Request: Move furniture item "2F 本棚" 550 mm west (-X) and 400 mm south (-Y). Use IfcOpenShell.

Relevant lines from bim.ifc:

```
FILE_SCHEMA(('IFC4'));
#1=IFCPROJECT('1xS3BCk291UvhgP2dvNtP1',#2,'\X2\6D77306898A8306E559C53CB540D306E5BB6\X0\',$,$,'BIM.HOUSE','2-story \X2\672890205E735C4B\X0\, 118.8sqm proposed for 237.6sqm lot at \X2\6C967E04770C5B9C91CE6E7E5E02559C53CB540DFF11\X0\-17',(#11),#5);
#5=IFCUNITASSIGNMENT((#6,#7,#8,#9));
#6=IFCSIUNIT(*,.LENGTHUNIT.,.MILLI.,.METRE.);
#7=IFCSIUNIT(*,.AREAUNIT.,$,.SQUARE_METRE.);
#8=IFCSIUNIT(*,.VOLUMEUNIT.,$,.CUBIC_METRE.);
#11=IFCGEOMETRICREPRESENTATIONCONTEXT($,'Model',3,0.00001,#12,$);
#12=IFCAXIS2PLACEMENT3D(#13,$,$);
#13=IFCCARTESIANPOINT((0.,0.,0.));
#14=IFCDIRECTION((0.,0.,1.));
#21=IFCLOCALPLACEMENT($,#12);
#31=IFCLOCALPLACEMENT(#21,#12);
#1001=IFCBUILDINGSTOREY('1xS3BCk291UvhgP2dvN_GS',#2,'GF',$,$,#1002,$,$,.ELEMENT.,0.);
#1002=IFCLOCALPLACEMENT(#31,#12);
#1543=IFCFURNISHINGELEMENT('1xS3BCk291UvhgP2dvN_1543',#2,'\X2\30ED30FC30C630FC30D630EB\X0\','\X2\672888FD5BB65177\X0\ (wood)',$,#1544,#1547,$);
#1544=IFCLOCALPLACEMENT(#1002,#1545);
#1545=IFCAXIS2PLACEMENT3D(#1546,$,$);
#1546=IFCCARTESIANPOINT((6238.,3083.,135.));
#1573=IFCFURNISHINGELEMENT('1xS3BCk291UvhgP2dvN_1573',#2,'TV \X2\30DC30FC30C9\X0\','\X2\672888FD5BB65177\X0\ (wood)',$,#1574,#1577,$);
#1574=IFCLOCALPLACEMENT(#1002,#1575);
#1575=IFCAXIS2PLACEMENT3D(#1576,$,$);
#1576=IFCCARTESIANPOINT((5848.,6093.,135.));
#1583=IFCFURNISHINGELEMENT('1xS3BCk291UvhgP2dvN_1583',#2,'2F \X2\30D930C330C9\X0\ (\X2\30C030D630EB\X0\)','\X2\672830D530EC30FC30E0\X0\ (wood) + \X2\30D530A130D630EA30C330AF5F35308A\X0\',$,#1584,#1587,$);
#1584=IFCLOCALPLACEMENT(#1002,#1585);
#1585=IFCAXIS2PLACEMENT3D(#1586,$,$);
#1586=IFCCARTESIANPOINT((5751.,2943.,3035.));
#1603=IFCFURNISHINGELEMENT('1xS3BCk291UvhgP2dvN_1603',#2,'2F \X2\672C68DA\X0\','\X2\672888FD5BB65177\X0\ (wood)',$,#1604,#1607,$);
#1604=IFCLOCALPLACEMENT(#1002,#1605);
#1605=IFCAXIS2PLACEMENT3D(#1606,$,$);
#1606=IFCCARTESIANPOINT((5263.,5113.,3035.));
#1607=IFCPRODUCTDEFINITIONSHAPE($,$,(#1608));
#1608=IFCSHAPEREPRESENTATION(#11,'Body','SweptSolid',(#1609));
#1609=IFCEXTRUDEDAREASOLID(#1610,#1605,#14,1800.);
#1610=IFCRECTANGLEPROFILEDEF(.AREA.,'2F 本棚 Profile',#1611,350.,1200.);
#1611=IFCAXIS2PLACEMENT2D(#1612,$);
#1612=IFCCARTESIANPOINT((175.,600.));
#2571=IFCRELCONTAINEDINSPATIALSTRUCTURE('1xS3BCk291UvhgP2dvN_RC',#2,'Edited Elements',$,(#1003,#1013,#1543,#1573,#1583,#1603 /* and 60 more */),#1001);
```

```python
import ifcopenshell
import ifcopenshell.api.geometry
import ifcopenshell.util.placement
import ifcopenshell.util.unit

model = ifcopenshell.open("bim.ifc")
unit_scale = ifcopenshell.util.unit.calculate_unit_scale(model)

item = model.by_guid("1xS3BCk291UvhgP2dvN_1603")
matrix = ifcopenshell.util.placement.get_local_placement(item.ObjectPlacement)
matrix[0, 3] -= 0.55 / unit_scale
matrix[1, 3] -= 0.4 / unit_scale
ifcopenshell.api.geometry.edit_object_placement(model, product=item, matrix=matrix, is_si=False)

print(ifcopenshell.util.placement.get_local_placement(item.ObjectPlacement).round(3) + 0.0)

model.write("bim_rev.ifc")
```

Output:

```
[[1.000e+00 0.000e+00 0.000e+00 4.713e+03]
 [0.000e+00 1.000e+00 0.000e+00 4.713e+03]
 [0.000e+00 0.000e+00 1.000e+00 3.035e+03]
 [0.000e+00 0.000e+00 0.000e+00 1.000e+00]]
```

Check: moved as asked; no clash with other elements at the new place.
